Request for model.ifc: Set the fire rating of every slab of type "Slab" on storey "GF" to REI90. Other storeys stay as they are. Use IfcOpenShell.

First a look at what the model holds.

```python
import ifcopenshell
import ifcopenshell.util.element

model = ifcopenshell.open("model.ifc")
print(model.schema)
storey = next(s for s in model.by_type("IfcBuildingStorey") if s.Name == "GF")
slabs = [e for e in ifcopenshell.util.element.get_decomposition(storey) if e.is_a("IfcSlab")]
seen = {}
for e in slabs:
    element_type = ifcopenshell.util.element.get_type(e)
    key = (element_type.Name if element_type != e and element_type else None, ifcopenshell.util.element.get_pset(e, "Pset_SlabCommon", "FireRating"))
    seen[key] = seen.get(key, 0) + 1
for (name, value), count in sorted(seen.items(), key=str):
    print(count, "x", name, "|", value)
```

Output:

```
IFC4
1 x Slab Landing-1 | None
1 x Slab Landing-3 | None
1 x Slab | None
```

```python
import ifcopenshell
import ifcopenshell.api.pset
import ifcopenshell.util.element

model = ifcopenshell.open("model.ifc")

storey = next(s for s in model.by_type("IfcBuildingStorey") if s.Name == "GF")
slabs = [e for e in ifcopenshell.util.element.get_decomposition(storey) if e.is_a("IfcSlab")]

count = 0
for e in slabs:
    element_type = ifcopenshell.util.element.get_type(e)
    if element_type in (None, e) or element_type.Name != "Slab":
        continue
    # add_pset returns the element's existing set when there is one.
    pset = ifcopenshell.api.pset.add_pset(model, product=e, name="Pset_SlabCommon")
    ifcopenshell.api.pset.edit_pset(model, pset=pset, properties={"FireRating": "REI90"})
    count += 1

print(count, "slabs updated")

model.write("model_updated.ifc")
```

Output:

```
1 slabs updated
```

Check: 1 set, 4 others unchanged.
